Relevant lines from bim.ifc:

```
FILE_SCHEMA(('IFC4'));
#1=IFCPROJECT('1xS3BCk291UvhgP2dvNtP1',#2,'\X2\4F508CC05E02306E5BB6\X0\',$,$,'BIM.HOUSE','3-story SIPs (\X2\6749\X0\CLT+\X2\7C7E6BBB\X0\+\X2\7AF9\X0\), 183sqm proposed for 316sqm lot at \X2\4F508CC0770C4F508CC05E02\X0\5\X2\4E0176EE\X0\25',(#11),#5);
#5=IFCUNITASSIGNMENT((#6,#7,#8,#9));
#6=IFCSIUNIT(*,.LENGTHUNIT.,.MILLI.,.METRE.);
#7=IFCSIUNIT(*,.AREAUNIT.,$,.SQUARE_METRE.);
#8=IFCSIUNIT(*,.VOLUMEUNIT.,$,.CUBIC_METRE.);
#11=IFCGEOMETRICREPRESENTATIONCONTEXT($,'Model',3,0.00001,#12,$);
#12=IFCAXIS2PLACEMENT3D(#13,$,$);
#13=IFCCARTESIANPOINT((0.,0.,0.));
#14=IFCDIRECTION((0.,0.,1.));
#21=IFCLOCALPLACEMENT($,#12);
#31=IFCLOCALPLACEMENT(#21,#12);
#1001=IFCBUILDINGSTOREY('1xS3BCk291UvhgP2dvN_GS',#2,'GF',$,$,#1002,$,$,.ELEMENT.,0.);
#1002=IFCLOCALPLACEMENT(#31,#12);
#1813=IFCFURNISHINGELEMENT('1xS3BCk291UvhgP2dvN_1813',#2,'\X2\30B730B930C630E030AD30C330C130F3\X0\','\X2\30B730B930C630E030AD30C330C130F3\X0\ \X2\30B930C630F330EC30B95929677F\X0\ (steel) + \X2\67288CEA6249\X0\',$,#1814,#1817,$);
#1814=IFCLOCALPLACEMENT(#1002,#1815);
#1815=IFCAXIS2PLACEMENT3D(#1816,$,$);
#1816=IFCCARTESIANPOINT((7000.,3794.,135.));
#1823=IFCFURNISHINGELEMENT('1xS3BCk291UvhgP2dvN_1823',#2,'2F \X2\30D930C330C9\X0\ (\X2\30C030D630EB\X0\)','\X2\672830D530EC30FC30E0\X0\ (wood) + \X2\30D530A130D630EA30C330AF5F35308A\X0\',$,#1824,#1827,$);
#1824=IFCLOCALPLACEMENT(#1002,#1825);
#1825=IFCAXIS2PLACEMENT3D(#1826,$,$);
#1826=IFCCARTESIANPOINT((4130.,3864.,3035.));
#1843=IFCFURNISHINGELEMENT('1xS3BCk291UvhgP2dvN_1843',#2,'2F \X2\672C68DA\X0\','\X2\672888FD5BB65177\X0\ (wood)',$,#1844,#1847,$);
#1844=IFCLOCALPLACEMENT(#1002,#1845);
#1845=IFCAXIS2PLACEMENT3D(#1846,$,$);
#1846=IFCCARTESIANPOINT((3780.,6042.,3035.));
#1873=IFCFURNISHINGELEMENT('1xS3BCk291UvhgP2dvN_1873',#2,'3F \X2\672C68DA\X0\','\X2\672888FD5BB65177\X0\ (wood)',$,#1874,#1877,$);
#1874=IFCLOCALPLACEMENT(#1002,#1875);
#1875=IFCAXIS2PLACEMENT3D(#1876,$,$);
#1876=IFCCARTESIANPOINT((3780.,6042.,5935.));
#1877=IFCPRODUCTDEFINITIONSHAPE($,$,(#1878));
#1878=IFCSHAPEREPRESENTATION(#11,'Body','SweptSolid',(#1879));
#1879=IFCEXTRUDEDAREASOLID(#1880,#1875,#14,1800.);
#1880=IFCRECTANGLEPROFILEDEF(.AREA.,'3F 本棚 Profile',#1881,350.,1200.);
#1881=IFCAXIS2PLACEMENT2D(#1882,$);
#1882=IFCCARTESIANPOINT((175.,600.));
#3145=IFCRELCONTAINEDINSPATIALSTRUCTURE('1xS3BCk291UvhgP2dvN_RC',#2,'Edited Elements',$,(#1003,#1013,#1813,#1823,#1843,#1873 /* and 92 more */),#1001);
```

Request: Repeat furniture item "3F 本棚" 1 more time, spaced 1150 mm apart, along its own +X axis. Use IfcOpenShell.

```python
import ifcopenshell
import ifcopenshell.api.geometry
import ifcopenshell.api.root
import ifcopenshell.util.element
import ifcopenshell.util.placement
import ifcopenshell.util.unit

model = ifcopenshell.open("bim.ifc")
unit_scale = ifcopenshell.util.unit.calculate_unit_scale(model)


def reuse_history(source, copy):
    """copy_class also copies each property set's owner history, people and application; keep the originals."""
    for rel in copy.IsDefinedBy:
        if rel.is_a("IfcRelDefinesByProperties") and (history := rel.RelatingPropertyDefinition.OwnerHistory):
            rel.RelatingPropertyDefinition.OwnerHistory = source.OwnerHistory
            ifcopenshell.util.element.remove_deep2(model, history)


source = model.by_id(1873)
base = ifcopenshell.util.placement.get_local_placement(source.ObjectPlacement)
step = base[:3, 0] * 1.15 / unit_scale

for i in range(1, 2):
    copy = ifcopenshell.api.root.copy_class(model, product=source)
    copy.Representation = ifcopenshell.util.element.copy_deep(
        model, source.Representation, exclude=["IfcGeometricRepresentationContext", "IfcRepresentationMap"]
    )
    reuse_history(source, copy)
    matrix = base.copy()
    matrix[:3, 3] += i * step
    print("added at", matrix[:3, 3].round(3) + 0.0)
    ifcopenshell.api.geometry.edit_object_placement(model, product=copy, matrix=matrix, is_si=False)

model.write("bim_v2.ifc")
```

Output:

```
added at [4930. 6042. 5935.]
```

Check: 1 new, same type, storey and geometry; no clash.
